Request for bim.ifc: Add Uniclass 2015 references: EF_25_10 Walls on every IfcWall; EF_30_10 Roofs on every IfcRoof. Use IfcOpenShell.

First a look at what the model holds.

```python
import ifcopenshell

model = ifcopenshell.open("bim.ifc")
print(model.schema)
print("classifications:", [c.Name for c in model.by_type("IfcClassification")])
for ifc_class in ("IfcDoor", "IfcRoof", "IfcStair", "IfcWall", "IfcWindow"):
    print(ifc_class, len(model.by_type(ifc_class)))
```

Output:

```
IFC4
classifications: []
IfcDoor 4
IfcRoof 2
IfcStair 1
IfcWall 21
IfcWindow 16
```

```python
import ifcopenshell
import ifcopenshell.api.classification

model = ifcopenshell.open("bim.ifc")

system = ifcopenshell.api.classification.add_classification(model, classification="Uniclass 2015")

codes = {
    "IfcWall": ("EF_25_10", "Walls"),
    "IfcRoof": ("EF_30_10", "Roofs"),
}
for ifc_class, (code, name) in codes.items():
    products = model.by_type(ifc_class)
    ifcopenshell.api.classification.add_reference(
        model, products=products, classification=system, identification=code, name=name
    )
    print(code, len(products))

model.write("bim_updated.ifc")
```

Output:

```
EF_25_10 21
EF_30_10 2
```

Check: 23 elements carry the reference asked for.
